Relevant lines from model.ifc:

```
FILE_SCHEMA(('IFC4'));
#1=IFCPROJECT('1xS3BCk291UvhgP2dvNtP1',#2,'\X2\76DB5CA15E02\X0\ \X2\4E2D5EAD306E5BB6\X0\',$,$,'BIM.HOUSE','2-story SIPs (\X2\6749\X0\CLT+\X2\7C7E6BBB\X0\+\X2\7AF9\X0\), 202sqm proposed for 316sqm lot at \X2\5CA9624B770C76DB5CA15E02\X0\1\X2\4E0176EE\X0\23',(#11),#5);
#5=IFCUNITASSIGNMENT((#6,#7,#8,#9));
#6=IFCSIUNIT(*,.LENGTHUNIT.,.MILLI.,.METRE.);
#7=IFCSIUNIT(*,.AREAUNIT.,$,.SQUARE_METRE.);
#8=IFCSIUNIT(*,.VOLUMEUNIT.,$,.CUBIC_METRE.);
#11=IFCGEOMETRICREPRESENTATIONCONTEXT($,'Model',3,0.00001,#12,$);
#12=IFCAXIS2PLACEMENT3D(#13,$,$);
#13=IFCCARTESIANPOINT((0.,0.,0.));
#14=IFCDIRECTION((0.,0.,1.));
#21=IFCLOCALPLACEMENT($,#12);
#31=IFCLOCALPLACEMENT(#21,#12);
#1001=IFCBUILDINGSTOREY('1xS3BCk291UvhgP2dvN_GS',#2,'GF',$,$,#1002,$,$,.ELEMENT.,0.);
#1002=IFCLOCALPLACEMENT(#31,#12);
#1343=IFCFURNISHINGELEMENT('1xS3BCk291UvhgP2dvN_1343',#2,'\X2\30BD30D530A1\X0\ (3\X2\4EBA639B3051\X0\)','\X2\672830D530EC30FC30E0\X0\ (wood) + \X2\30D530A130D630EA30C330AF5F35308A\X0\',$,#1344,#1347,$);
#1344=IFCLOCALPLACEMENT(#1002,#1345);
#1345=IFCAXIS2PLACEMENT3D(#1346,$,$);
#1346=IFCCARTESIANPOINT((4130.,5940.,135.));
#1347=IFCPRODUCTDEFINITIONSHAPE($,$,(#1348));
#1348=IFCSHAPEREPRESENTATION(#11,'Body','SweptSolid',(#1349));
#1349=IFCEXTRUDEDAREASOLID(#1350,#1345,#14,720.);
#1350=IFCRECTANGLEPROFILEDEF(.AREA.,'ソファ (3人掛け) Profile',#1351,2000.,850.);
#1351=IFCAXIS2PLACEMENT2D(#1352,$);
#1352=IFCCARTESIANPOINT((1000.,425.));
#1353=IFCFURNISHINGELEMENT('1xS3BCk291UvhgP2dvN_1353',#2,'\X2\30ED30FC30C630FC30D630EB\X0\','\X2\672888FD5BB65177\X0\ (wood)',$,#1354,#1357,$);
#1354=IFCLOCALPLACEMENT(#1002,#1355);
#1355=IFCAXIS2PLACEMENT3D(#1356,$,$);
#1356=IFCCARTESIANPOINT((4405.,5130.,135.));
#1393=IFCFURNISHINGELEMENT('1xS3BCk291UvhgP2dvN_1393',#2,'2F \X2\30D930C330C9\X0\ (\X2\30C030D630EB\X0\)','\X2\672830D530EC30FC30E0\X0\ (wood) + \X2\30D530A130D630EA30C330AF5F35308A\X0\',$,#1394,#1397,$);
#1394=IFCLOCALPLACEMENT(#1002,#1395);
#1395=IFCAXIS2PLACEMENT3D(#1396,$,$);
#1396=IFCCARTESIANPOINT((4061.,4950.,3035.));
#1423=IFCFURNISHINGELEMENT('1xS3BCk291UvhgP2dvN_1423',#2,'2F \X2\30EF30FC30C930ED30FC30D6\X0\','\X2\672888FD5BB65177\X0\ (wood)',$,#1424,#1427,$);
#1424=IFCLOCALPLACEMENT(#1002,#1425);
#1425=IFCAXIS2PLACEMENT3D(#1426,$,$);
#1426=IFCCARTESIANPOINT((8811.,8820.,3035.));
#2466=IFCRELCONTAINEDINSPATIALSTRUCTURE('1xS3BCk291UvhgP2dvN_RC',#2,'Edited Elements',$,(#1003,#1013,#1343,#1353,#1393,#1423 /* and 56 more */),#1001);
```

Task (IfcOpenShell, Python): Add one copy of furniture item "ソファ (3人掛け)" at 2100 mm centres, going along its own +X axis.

```python
import ifcopenshell
import ifcopenshell.api.geometry
import ifcopenshell.api.root
import ifcopenshell.util.element
import ifcopenshell.util.placement
import ifcopenshell.util.unit

model = ifcopenshell.open("model.ifc")
unit_scale = ifcopenshell.util.unit.calculate_unit_scale(model)


def reuse_history(source, copy):
    """copy_class also copies each property set's owner history, people and application; keep the originals."""
    for rel in copy.IsDefinedBy:
        if rel.is_a("IfcRelDefinesByProperties") and (history := rel.RelatingPropertyDefinition.OwnerHistory):
            rel.RelatingPropertyDefinition.OwnerHistory = source.OwnerHistory
            ifcopenshell.util.element.remove_deep2(model, history)


source = model.by_guid("1xS3BCk291UvhgP2dvN_1343")
base = ifcopenshell.util.placement.get_local_placement(source.ObjectPlacement)
step = base[:3, 0] * 2.1 / unit_scale

for i in range(1, 2):
    copy = ifcopenshell.api.root.copy_class(model, product=source)
    copy.Representation = ifcopenshell.util.element.copy_deep(
        model, source.Representation, exclude=["IfcGeometricRepresentationContext", "IfcRepresentationMap"]
    )
    reuse_history(source, copy)
    matrix = base.copy()
    matrix[:3, 3] += i * step
    print("added at", matrix[:3, 3].round(3) + 0.0)
    ifcopenshell.api.geometry.edit_object_placement(model, product=copy, matrix=matrix, is_si=False)

model.write("model_updated.ifc")
```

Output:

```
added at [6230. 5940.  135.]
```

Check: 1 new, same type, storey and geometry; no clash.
